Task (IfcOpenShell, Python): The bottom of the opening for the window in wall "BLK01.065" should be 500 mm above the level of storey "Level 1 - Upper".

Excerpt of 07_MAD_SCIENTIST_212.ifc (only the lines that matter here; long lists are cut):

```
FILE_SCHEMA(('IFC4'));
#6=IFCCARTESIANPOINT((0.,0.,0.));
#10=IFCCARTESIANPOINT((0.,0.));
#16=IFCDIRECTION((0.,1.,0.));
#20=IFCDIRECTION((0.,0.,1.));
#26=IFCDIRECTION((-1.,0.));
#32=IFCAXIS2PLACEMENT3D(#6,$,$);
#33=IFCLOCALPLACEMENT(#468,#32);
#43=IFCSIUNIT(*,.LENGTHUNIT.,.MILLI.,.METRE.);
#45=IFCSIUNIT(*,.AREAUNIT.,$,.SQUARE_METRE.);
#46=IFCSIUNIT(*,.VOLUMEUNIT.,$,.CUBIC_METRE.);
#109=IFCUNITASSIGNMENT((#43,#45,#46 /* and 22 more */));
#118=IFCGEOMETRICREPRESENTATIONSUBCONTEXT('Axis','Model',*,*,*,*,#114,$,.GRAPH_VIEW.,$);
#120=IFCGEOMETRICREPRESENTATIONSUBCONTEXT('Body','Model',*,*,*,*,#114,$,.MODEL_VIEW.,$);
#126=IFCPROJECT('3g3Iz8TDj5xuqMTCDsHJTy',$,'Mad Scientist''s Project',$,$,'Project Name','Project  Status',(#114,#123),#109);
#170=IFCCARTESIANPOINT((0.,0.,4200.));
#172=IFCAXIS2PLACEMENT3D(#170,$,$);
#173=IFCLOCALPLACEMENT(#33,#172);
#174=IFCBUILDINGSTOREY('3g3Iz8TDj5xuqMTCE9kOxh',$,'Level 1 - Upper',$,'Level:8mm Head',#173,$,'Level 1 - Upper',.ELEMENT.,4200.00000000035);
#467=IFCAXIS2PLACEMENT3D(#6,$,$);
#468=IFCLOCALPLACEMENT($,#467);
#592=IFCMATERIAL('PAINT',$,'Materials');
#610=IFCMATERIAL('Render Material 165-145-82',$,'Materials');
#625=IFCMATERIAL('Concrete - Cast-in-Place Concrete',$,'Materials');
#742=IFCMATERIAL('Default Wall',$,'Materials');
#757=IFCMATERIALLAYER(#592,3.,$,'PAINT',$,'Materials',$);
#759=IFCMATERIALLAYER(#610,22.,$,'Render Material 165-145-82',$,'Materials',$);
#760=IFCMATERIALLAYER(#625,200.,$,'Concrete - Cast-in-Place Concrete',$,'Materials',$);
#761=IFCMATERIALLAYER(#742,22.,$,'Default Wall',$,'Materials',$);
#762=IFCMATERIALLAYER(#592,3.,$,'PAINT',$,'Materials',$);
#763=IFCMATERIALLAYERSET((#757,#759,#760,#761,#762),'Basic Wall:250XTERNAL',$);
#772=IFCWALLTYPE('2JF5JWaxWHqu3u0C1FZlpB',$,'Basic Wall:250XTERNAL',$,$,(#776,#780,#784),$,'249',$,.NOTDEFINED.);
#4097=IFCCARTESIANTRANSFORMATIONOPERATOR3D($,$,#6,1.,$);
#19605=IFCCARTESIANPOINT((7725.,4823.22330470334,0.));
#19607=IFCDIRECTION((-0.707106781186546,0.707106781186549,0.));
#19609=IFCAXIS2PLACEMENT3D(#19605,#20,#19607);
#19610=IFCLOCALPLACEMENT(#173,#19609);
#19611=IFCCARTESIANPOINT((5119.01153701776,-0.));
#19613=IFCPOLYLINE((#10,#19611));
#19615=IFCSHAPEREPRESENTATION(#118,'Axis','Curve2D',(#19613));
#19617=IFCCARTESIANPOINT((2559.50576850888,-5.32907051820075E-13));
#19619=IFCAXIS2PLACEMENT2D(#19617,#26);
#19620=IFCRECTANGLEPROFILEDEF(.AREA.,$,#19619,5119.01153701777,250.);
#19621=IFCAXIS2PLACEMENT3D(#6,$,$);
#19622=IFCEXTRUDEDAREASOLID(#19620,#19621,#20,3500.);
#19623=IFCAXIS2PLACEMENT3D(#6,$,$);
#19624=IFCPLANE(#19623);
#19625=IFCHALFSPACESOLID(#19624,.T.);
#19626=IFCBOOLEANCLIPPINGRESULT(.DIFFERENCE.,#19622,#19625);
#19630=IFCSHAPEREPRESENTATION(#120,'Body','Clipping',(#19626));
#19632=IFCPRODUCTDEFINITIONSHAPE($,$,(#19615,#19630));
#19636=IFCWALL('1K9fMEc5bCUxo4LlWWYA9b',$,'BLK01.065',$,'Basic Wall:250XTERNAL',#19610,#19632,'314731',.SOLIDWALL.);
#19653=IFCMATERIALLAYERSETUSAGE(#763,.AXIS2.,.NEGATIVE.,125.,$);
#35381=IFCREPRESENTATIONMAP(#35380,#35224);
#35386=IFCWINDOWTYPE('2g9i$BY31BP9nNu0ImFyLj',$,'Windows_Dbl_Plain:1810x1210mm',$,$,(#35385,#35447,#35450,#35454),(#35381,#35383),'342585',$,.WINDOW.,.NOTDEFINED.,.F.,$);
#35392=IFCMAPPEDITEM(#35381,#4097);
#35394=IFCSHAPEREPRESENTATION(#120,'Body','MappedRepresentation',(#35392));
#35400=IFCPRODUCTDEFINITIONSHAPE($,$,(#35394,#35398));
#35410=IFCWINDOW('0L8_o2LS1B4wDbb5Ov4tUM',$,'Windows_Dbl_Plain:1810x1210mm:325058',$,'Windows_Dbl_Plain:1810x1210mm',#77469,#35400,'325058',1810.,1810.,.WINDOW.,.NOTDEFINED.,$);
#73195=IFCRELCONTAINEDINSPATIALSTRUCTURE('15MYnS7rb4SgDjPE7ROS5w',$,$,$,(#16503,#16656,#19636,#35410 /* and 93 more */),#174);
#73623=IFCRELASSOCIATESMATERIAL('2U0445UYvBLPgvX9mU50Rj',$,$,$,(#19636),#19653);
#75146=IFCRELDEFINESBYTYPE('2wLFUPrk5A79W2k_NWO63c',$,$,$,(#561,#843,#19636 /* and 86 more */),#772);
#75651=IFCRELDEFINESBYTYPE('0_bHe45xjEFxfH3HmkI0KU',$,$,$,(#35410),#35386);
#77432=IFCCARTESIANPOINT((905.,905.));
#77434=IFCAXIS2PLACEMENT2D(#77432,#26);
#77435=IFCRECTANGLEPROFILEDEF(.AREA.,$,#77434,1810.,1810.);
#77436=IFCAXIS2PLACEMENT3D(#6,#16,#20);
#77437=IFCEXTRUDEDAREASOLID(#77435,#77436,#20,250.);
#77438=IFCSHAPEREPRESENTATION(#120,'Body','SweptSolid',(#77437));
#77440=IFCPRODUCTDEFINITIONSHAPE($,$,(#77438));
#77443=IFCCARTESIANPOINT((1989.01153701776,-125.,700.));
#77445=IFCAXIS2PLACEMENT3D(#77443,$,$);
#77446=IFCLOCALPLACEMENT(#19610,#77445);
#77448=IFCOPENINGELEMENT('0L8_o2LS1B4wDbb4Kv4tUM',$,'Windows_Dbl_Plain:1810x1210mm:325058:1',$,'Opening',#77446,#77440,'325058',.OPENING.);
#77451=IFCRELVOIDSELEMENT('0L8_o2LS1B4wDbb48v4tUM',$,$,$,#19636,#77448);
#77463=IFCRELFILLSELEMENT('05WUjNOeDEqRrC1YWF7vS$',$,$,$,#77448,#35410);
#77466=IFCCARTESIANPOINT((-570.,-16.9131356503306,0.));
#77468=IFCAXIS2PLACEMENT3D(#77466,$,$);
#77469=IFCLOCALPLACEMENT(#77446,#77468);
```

```python
import numpy as np
import ifcopenshell
import ifcopenshell.api.geometry
import ifcopenshell.geom
import ifcopenshell.util.element
import ifcopenshell.util.placement
import ifcopenshell.util.shape
import ifcopenshell.util.unit

model = ifcopenshell.open("07_MAD_SCIENTIST_212.ifc")
unit_scale = ifcopenshell.util.unit.calculate_unit_scale(model)

window = model.by_guid("0L8_o2LS1B4wDbb5Ov4tUM")
opening = window.FillsVoids[0].RelatingOpeningElement
storey = ifcopenshell.util.element.get_container(window, ifc_class="IfcBuildingStorey")
level = ifcopenshell.util.placement.get_local_placement(storey.ObjectPlacement)[2, 3]

# The opening's origin need not be at the sill, so measure its lowest point.
shape = ifcopenshell.geom.create_shape(ifcopenshell.geom.settings(), opening)
bottom = ifcopenshell.util.shape.get_shape_bottom_elevation(shape, shape.geometry) / unit_scale
dz = level + 0.5 / unit_scale - bottom

shift = np.array([0.0, 0.0, dz])
# The window is placed relative to its opening, so it follows when the opening moves.
matrix = ifcopenshell.util.placement.get_local_placement(opening.ObjectPlacement)
matrix[:3, 3] += shift
ifcopenshell.api.geometry.edit_object_placement(
    model, product=opening, matrix=matrix, is_si=False, should_transform_children=True
)

print(f"moved by {dz * unit_scale:+.3f} m")

model.write("07_MAD_SCIENTIST_212_v2.ifc")
```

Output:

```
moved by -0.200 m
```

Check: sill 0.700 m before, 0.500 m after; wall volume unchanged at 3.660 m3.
